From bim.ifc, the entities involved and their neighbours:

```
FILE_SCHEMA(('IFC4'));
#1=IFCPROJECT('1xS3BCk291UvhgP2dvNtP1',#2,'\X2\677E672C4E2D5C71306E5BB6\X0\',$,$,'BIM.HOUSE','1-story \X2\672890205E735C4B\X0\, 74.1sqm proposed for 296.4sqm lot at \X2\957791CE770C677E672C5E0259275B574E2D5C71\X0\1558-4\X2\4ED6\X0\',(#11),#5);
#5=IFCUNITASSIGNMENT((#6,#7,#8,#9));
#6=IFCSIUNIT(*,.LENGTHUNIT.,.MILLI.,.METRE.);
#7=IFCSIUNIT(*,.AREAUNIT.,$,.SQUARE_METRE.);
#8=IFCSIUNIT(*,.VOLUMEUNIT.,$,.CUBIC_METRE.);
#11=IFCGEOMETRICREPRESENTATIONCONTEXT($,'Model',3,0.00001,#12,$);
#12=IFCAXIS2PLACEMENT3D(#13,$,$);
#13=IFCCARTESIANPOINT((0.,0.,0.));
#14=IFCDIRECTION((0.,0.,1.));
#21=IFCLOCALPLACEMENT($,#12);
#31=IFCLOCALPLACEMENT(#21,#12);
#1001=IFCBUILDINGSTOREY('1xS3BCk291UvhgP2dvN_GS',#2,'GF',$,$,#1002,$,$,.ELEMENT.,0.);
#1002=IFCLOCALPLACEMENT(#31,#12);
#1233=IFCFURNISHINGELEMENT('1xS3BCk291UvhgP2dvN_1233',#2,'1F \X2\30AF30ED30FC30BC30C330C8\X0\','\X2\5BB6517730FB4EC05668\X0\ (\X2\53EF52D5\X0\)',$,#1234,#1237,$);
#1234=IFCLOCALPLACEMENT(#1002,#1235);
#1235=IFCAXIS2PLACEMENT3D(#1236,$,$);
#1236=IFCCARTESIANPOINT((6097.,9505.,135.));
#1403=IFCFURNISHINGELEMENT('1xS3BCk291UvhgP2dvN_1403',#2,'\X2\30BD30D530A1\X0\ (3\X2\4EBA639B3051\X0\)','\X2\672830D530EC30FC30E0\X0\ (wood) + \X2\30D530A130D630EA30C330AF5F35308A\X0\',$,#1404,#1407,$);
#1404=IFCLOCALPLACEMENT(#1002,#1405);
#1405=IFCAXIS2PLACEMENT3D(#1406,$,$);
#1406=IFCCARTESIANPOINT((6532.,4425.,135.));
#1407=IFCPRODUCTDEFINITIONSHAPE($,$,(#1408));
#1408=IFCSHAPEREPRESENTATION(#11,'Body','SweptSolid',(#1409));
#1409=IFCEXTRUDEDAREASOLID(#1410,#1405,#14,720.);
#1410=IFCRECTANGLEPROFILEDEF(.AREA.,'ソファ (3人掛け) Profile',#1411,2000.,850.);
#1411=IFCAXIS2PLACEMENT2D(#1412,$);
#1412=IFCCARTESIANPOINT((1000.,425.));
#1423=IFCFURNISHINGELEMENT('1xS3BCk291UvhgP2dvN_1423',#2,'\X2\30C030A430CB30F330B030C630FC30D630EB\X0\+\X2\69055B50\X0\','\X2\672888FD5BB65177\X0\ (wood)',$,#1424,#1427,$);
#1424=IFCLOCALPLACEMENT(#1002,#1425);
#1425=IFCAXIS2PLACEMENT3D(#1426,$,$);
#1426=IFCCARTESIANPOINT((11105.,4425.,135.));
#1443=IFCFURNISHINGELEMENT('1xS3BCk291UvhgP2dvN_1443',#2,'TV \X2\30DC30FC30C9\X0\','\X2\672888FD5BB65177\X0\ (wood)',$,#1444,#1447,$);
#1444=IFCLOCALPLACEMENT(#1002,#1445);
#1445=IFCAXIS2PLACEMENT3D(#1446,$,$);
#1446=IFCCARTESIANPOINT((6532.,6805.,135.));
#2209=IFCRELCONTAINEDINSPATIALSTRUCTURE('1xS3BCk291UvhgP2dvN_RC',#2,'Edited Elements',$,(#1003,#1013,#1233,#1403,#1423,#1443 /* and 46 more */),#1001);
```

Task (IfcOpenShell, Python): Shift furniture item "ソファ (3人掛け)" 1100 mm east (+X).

```python
import ifcopenshell
import ifcopenshell.api.geometry
import ifcopenshell.util.placement

model = ifcopenshell.open("bim.ifc")

item = model.by_guid("1xS3BCk291UvhgP2dvN_1403")
matrix = ifcopenshell.util.placement.get_local_placement(item.ObjectPlacement)
matrix[0, 3] += 1100.0
ifcopenshell.api.geometry.edit_object_placement(model, product=item, matrix=matrix, is_si=False)

print(ifcopenshell.util.placement.get_local_placement(item.ObjectPlacement).round(3) + 0.0)

model.write("bim_v2.ifc")
```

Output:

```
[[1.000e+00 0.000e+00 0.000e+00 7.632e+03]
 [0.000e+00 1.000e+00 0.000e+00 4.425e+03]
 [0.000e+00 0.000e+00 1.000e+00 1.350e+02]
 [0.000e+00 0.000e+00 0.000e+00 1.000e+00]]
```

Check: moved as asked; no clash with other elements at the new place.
